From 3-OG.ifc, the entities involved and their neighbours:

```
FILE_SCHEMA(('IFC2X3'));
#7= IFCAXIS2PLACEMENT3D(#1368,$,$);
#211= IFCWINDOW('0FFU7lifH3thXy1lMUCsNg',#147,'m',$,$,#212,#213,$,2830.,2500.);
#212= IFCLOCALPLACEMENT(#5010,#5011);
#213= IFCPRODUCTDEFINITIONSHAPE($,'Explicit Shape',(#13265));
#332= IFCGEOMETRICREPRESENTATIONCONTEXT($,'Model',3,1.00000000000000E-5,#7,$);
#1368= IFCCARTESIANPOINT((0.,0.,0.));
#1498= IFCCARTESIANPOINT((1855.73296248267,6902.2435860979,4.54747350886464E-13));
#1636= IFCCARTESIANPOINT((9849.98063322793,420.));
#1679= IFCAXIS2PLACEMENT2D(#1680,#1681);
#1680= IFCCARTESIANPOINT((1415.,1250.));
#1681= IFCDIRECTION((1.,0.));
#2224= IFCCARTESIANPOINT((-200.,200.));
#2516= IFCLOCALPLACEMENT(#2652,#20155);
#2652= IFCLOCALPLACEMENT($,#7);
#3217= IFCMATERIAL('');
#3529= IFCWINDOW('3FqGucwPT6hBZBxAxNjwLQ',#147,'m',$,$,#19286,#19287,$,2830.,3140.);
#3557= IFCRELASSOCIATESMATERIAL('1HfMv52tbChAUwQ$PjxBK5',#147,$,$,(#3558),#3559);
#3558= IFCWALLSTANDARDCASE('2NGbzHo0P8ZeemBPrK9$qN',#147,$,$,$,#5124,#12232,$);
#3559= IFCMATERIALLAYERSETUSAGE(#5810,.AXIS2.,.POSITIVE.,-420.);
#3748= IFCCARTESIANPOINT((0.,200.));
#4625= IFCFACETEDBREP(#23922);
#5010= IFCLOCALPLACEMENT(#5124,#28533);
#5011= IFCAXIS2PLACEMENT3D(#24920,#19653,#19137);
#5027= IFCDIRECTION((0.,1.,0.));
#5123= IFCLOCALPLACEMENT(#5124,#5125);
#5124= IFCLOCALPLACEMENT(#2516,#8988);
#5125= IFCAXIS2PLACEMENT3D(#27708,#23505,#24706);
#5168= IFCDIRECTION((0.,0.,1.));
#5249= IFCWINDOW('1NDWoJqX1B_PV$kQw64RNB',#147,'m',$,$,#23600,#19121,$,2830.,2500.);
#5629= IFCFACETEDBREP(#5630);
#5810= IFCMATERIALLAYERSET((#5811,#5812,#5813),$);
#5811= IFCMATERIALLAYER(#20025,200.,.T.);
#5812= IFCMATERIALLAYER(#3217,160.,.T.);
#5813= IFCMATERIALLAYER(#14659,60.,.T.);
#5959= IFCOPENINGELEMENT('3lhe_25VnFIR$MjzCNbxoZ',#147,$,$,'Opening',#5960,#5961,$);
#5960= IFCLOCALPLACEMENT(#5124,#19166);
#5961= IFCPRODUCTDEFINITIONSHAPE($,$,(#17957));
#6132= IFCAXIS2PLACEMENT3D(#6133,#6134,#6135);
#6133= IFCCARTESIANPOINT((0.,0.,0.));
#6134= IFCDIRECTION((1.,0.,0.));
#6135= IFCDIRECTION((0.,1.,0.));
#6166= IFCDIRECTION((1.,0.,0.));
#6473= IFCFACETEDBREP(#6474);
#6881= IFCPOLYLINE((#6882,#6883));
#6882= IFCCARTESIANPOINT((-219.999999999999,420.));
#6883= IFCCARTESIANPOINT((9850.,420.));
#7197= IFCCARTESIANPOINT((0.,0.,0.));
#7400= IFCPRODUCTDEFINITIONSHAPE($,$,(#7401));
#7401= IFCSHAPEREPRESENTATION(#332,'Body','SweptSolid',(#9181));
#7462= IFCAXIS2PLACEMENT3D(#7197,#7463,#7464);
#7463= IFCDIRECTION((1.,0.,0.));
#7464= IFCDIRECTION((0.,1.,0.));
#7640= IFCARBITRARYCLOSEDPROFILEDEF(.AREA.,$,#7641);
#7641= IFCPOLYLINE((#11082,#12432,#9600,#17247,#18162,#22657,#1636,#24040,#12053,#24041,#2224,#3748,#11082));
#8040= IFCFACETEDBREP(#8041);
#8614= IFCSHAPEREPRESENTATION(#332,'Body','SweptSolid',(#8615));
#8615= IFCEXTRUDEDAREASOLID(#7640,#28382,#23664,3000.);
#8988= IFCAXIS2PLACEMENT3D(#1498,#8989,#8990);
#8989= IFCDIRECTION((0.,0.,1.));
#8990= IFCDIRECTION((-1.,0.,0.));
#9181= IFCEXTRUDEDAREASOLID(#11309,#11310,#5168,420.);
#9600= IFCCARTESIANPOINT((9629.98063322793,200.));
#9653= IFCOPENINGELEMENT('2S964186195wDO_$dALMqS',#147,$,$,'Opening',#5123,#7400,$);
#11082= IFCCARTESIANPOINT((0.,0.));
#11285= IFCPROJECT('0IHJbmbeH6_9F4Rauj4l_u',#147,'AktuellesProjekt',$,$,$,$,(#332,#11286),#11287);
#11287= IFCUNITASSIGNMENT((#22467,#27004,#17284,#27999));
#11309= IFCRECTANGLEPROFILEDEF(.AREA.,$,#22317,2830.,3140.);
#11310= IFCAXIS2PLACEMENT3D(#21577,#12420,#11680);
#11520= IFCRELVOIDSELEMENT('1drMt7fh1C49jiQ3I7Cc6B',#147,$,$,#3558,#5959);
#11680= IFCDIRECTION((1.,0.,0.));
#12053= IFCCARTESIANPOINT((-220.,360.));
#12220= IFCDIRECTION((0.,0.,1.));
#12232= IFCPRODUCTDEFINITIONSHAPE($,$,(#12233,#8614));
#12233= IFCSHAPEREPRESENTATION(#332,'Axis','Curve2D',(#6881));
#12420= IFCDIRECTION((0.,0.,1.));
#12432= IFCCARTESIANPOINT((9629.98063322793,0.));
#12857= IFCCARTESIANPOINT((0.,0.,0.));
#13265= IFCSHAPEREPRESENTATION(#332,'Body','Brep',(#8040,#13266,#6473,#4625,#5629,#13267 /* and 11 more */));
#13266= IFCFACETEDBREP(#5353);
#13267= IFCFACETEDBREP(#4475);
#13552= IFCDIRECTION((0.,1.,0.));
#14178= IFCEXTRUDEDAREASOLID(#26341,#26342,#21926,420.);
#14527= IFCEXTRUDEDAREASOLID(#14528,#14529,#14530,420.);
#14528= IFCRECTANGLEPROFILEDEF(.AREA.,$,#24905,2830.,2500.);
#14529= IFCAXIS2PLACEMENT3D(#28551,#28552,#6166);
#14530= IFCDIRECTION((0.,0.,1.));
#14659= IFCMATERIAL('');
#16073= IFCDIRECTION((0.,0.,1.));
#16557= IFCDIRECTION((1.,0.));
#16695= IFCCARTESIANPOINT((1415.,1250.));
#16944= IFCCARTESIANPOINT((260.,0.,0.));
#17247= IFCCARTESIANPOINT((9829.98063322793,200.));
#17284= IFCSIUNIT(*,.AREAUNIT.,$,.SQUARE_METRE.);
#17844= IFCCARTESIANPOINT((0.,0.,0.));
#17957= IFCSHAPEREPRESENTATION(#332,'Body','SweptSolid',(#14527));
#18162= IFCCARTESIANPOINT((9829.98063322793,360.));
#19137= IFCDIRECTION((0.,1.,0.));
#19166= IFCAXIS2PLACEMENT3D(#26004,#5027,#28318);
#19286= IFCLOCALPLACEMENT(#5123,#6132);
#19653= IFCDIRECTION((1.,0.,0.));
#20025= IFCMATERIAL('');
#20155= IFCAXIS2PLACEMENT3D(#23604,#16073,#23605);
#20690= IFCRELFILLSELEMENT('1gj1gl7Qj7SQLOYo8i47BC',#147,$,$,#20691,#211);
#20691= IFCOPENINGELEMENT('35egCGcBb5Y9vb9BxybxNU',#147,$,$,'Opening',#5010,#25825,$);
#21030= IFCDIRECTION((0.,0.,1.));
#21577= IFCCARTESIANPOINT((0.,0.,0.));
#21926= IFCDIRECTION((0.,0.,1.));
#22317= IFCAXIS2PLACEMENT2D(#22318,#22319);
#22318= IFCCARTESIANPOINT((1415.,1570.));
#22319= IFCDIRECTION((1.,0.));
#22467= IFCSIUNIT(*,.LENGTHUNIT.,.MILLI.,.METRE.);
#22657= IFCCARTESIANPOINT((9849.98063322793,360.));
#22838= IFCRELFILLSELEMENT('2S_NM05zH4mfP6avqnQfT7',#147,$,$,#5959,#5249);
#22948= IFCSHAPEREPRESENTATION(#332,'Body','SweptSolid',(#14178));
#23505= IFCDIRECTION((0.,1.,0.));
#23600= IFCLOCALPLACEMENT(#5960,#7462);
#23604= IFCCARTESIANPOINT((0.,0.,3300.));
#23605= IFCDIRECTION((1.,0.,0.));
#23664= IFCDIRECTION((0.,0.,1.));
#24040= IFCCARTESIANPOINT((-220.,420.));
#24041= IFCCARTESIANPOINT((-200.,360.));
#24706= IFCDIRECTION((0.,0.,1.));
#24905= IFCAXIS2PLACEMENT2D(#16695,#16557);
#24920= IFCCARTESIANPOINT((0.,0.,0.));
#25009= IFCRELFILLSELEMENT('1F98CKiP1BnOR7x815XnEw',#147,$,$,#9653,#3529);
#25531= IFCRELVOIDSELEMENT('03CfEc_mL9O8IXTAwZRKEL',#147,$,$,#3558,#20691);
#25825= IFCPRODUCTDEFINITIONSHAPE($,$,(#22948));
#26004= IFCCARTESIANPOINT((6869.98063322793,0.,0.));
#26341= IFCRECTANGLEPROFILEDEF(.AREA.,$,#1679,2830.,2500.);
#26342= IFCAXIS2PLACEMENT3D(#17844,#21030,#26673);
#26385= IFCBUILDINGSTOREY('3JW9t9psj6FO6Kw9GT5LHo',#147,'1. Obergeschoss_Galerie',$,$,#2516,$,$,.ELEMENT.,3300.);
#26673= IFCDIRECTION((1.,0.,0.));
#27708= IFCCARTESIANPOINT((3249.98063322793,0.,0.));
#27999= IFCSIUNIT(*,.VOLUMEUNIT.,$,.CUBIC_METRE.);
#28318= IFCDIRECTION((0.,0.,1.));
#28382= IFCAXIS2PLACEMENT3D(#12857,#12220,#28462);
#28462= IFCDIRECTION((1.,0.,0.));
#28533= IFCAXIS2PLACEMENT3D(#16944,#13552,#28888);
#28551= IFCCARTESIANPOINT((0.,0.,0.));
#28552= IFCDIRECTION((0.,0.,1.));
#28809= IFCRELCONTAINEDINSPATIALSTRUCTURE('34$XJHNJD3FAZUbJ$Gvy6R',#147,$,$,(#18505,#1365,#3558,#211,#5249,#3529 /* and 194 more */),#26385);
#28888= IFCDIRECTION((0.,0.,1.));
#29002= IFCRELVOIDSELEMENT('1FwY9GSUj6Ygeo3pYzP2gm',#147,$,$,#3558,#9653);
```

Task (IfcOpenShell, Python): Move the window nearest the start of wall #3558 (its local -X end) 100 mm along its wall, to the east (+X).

```python
import ifcopenshell
import ifcopenshell.api.geometry
import ifcopenshell.util.placement
import ifcopenshell.util.unit

model = ifcopenshell.open("3-OG.ifc")
unit_scale = ifcopenshell.util.unit.calculate_unit_scale(model)

window = model.by_guid("0FFU7lifH3thXy1lMUCsNg")
opening = window.FillsVoids[0].RelatingOpeningElement
wall = opening.VoidsElements[0].RelatingBuildingElement

wall_matrix = ifcopenshell.util.placement.get_local_placement(wall.ObjectPlacement)
shift = wall_matrix[:3, 0] * -0.1 / unit_scale
before = ifcopenshell.util.placement.get_local_placement(window.ObjectPlacement)[:3, 3].copy()

# The window is placed relative to its opening, so it follows when the opening moves.
matrix = ifcopenshell.util.placement.get_local_placement(opening.ObjectPlacement)
matrix[:3, 3] += shift
ifcopenshell.api.geometry.edit_object_placement(
    model, product=opening, matrix=matrix, is_si=False, should_transform_children=True
)

after = ifcopenshell.util.placement.get_local_placement(window.ObjectPlacement)[:3, 3]
print("window moved by", (after - before).round(3) + 0.0)

model.write("3-OG_edited.ifc")
```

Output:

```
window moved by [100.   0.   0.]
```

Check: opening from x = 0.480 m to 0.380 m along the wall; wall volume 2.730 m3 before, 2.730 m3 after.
